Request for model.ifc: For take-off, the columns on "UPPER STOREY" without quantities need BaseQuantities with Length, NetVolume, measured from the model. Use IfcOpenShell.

First a look at what the model holds.

```python
import ifcopenshell
import ifcopenshell.util.element
import ifcopenshell.util.unit

model = ifcopenshell.open("model.ifc")
print(model.schema)
for unit_type in ("LENGTHUNIT", "AREAUNIT", "VOLUMEUNIT"):
    print(unit_type, ifcopenshell.util.unit.calculate_unit_scale(model, unit_type))
storey = next(s for s in model.by_type("IfcBuildingStorey") if s.Name == "UPPER STOREY")
columns = [e for e in ifcopenshell.util.element.get_decomposition(storey) if e.is_a("IfcColumn")]
for e in sorted(columns, key=lambda e: e.id()):
    print(e.id(), e.is_a(), e.Name, list(ifcopenshell.util.element.get_psets(e, qtos_only=True)), sep=" | ")
```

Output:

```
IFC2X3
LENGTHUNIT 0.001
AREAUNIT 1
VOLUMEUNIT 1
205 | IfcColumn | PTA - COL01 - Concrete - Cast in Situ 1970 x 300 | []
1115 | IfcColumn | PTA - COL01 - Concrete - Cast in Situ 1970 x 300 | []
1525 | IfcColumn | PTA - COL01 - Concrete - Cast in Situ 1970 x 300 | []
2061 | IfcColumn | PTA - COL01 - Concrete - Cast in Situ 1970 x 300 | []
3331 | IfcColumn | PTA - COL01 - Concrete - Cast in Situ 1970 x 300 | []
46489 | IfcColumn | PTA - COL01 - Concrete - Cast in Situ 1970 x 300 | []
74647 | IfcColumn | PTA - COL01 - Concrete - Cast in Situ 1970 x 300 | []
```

```python
import ifcopenshell
import ifcopenshell.api.pset
import ifcopenshell.geom
import ifcopenshell.util.element
import ifcopenshell.util.shape
import ifcopenshell.util.unit

model = ifcopenshell.open("model.ifc")
unit_scale = ifcopenshell.util.unit.calculate_unit_scale(model)
volume_scale = ifcopenshell.util.unit.calculate_unit_scale(model, "VOLUMEUNIT")
settings = ifcopenshell.geom.settings()

storey = next(s for s in model.by_type("IfcBuildingStorey") if s.Name == "UPPER STOREY")
columns = [e for e in ifcopenshell.util.element.get_decomposition(storey) if e.is_a("IfcColumn")]

for e in sorted(columns, key=lambda e: e.id()):
    if ifcopenshell.util.element.get_psets(e, qtos_only=True, should_inherit=False):
        continue
    # Geometry comes back in metres, in the element's own axes.
    shape = ifcopenshell.geom.create_shape(settings, e)
    values = {
        "Length": ifcopenshell.util.shape.get_z(shape.geometry) / unit_scale,
        "NetVolume": ifcopenshell.util.shape.get_volume(shape.geometry) / volume_scale,
    }
    qto = ifcopenshell.api.pset.add_qto(model, product=e, name="BaseQuantities")
    ifcopenshell.api.pset.edit_qto(model, qto=qto, properties=values)
    print(e.id(), {k: round(v, 3) for k, v in values.items()})

model.write("model_v2.ifc")
```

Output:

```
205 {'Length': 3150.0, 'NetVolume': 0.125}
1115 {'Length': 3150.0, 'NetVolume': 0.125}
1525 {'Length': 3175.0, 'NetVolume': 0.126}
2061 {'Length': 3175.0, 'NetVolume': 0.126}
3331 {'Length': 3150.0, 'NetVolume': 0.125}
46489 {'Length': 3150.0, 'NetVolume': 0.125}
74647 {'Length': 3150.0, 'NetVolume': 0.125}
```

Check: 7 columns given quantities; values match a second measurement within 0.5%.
